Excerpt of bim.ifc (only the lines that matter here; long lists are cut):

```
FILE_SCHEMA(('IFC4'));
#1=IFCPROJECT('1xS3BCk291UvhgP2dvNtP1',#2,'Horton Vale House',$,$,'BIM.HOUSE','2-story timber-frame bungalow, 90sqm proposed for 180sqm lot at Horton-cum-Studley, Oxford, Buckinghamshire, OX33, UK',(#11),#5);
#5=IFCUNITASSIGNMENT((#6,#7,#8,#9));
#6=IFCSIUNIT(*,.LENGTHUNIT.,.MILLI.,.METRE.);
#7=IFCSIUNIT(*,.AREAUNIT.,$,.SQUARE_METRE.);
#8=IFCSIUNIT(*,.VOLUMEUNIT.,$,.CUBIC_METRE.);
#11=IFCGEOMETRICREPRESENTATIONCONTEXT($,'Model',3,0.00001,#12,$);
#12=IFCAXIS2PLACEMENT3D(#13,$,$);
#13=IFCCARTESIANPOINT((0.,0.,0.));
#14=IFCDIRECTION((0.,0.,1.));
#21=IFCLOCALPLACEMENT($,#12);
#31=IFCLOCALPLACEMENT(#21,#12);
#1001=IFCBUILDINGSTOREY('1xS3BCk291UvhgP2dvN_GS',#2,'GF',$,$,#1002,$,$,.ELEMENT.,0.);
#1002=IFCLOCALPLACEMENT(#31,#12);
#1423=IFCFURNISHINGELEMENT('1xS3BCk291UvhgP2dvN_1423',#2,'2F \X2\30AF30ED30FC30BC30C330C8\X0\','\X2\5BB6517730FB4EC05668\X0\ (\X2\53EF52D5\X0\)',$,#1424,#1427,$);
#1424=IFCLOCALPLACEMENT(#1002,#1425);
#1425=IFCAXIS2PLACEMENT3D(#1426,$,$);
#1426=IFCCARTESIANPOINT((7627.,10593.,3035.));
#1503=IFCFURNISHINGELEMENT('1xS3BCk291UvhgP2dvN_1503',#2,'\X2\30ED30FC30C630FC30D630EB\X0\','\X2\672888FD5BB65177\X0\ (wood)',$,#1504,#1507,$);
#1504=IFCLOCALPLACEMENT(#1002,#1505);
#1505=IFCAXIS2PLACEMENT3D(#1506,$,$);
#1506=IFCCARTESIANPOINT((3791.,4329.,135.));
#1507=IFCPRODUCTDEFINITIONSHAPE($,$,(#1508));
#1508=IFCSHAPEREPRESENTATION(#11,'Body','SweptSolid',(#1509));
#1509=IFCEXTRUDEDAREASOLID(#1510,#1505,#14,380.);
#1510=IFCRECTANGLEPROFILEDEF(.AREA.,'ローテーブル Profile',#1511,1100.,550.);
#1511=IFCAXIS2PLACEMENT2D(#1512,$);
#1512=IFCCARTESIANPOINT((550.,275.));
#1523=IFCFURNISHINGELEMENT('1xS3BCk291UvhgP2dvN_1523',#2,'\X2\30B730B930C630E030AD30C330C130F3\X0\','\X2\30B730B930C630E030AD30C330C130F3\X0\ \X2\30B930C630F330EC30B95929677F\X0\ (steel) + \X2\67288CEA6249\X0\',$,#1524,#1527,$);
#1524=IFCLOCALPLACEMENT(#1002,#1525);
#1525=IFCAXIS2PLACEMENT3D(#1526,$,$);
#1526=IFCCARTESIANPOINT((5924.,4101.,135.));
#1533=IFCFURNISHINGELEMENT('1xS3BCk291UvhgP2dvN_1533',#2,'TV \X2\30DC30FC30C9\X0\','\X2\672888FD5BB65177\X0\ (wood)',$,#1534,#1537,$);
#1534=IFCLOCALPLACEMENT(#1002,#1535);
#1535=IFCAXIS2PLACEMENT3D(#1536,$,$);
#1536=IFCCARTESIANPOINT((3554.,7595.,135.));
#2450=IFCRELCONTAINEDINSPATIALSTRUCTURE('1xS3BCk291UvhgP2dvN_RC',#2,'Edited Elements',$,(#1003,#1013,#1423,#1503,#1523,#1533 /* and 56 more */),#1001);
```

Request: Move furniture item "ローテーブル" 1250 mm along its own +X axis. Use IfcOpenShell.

```python
import ifcopenshell
import ifcopenshell.api.geometry
import ifcopenshell.util.placement

model = ifcopenshell.open("bim.ifc")

item = model.by_guid("1xS3BCk291UvhgP2dvN_1503")
matrix = ifcopenshell.util.placement.get_local_placement(item.ObjectPlacement)
matrix[:3, 3] += matrix[:3, 0] * 1250.0
ifcopenshell.api.geometry.edit_object_placement(model, product=item, matrix=matrix, is_si=False)

print(ifcopenshell.util.placement.get_local_placement(item.ObjectPlacement).round(3) + 0.0)

model.write("bim_edited.ifc")
```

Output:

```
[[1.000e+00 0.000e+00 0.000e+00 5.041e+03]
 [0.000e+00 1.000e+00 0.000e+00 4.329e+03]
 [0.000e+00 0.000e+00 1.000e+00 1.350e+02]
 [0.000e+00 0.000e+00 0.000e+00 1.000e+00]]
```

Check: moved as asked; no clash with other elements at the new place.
